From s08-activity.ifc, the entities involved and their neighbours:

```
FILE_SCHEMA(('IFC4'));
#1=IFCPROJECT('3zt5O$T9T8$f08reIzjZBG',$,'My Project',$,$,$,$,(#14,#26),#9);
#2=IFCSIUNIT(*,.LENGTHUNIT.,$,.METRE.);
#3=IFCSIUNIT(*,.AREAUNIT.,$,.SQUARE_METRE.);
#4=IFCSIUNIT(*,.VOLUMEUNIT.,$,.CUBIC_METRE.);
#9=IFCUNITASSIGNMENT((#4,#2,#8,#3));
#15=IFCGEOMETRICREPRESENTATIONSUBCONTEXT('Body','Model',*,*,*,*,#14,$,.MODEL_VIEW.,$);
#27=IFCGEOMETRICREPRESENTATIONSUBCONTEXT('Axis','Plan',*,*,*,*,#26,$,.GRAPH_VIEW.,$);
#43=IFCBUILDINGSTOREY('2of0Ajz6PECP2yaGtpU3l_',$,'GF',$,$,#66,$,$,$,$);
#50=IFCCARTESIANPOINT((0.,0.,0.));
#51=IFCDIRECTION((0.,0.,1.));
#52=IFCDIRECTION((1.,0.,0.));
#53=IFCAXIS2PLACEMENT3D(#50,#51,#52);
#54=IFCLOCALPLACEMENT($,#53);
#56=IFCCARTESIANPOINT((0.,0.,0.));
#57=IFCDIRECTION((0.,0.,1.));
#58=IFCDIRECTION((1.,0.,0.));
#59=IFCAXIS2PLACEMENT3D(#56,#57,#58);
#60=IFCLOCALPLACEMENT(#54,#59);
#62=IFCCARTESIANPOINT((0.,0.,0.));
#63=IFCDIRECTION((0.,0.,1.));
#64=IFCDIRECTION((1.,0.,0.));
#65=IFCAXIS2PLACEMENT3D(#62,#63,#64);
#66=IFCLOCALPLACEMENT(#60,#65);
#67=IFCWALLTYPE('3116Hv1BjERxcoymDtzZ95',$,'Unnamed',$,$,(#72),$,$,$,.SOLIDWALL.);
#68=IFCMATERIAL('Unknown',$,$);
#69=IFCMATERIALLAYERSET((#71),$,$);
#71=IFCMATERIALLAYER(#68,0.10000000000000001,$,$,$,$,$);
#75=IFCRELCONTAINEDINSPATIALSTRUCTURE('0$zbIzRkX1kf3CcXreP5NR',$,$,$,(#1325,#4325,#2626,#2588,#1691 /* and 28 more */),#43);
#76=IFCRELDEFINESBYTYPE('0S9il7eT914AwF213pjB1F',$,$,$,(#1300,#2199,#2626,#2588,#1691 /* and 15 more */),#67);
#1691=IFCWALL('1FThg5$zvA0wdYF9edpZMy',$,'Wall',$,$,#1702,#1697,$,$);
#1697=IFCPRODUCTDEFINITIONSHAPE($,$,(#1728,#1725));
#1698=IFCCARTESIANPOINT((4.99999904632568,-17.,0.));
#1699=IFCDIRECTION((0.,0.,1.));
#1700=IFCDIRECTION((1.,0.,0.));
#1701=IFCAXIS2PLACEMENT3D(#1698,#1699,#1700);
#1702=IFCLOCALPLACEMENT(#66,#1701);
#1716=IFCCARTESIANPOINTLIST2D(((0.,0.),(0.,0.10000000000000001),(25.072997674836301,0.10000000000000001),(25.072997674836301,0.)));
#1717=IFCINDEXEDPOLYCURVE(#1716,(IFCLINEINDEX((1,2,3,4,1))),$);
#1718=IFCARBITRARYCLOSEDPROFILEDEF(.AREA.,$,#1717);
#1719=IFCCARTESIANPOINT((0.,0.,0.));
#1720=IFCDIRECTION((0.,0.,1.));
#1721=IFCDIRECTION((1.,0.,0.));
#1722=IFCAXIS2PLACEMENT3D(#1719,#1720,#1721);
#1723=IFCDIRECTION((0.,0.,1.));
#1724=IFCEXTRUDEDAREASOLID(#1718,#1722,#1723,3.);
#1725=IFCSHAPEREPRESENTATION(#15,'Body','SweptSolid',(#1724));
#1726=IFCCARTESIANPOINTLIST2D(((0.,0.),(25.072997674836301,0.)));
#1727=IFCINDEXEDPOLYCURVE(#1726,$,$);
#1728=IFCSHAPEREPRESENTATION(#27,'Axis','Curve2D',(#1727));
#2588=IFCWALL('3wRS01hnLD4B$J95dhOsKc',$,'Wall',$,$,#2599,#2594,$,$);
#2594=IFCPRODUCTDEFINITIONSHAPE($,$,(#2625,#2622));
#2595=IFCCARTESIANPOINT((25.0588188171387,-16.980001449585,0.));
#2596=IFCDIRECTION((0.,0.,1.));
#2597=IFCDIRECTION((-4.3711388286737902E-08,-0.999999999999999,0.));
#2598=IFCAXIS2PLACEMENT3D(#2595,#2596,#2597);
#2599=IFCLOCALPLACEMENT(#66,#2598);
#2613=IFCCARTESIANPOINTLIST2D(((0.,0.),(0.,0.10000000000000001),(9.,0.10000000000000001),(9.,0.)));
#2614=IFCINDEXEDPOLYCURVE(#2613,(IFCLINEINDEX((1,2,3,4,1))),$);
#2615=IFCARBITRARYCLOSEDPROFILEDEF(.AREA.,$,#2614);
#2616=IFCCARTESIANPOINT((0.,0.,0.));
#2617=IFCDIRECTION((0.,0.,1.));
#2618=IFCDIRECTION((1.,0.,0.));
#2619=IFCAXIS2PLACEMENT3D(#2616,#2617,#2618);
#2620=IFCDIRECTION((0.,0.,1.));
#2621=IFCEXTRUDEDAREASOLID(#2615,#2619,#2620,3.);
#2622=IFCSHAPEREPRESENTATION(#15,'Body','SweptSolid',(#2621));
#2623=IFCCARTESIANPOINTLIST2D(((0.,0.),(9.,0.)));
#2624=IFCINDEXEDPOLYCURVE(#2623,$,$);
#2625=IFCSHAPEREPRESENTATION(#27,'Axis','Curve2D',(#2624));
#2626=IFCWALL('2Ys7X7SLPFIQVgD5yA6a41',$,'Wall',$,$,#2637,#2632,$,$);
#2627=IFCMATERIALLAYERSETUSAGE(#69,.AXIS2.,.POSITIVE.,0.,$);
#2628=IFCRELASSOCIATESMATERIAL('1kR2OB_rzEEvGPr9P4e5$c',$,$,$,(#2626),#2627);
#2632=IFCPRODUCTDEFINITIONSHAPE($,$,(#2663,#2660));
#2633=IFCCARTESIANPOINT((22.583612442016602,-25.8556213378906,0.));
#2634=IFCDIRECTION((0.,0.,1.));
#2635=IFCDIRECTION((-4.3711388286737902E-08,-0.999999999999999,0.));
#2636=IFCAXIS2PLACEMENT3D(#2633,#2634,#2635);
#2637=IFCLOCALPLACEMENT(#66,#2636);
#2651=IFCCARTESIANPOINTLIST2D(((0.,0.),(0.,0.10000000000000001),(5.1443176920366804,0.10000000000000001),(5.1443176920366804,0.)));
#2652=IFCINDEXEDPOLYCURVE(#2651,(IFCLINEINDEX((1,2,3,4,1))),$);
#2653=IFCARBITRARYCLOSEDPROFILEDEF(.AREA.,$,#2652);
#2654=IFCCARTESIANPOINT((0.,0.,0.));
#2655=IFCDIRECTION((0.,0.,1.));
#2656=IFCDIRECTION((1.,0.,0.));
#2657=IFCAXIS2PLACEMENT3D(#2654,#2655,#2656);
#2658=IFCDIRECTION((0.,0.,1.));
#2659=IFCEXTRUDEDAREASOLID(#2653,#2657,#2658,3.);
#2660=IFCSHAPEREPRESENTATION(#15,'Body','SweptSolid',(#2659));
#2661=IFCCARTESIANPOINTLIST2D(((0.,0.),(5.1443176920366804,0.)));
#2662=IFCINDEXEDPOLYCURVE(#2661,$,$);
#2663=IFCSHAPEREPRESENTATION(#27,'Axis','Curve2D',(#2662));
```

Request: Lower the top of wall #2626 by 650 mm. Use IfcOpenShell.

```python
import ifcopenshell
import ifcopenshell.geom
import ifcopenshell.util.representation
import ifcopenshell.util.shape
import ifcopenshell.util.unit

model = ifcopenshell.open("s08-activity.ifc")
unit_scale = ifcopenshell.util.unit.calculate_unit_scale(model)
settings = ifcopenshell.geom.settings()


def volume(element):
    """Net volume in cubic metres, openings subtracted."""
    shape = ifcopenshell.geom.create_shape(settings, element)
    return ifcopenshell.util.shape.get_volume(shape.geometry)


wall = model.by_id(2626)
before = volume(wall)

body = ifcopenshell.util.representation.get_representation(wall, "Model", "Body")
solid = body.Items[0]
old_height = solid.Depth
solid.Depth -= 0.65 / unit_scale
after = volume(wall)

print(f"height {old_height:g} -> {solid.Depth:g}, volume {before:.3f} -> {after:.3f} m3")

model.write("s08-activity_updated.ifc")
```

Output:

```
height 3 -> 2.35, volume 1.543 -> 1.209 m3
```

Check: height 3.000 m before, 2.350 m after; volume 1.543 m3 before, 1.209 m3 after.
